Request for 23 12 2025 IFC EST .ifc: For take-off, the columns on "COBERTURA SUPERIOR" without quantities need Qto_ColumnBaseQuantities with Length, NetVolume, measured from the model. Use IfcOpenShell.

First a look at what the model holds.

```python
import ifcopenshell
import ifcopenshell.util.element
import ifcopenshell.util.unit

model = ifcopenshell.open("23 12 2025 IFC EST .ifc")
print(model.schema)
for unit_type in ("LENGTHUNIT", "AREAUNIT", "VOLUMEUNIT"):
    print(unit_type, ifcopenshell.util.unit.calculate_unit_scale(model, unit_type))
storey = next(s for s in model.by_type("IfcBuildingStorey") if s.Name == "COBERTURA SUPERIOR")
columns = [e for e in ifcopenshell.util.element.get_decomposition(storey) if e.is_a("IfcColumn")]
for e in sorted(columns, key=lambda e: e.id()):
    print(e.id(), e.is_a(), e.Name, list(ifcopenshell.util.element.get_psets(e, qtos_only=True)), sep=" | ")
```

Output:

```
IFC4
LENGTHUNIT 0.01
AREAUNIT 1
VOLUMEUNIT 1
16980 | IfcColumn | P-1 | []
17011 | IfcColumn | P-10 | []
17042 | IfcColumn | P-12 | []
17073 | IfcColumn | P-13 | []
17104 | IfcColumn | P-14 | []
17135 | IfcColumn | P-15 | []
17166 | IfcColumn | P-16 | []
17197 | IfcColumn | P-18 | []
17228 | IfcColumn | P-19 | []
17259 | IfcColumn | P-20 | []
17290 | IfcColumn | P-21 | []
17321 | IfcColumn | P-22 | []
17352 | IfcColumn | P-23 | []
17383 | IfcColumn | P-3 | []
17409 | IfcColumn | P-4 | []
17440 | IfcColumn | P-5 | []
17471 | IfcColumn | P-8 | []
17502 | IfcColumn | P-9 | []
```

```python
import ifcopenshell
import ifcopenshell.api.pset
import ifcopenshell.geom
import ifcopenshell.util.element
import ifcopenshell.util.shape
import ifcopenshell.util.unit

model = ifcopenshell.open("23 12 2025 IFC EST .ifc")
unit_scale = ifcopenshell.util.unit.calculate_unit_scale(model)
volume_scale = ifcopenshell.util.unit.calculate_unit_scale(model, "VOLUMEUNIT")
settings = ifcopenshell.geom.settings()

storey = next(s for s in model.by_type("IfcBuildingStorey") if s.Name == "COBERTURA SUPERIOR")
columns = [e for e in ifcopenshell.util.element.get_decomposition(storey) if e.is_a("IfcColumn")]

for e in sorted(columns, key=lambda e: e.id()):
    if ifcopenshell.util.element.get_psets(e, qtos_only=True, should_inherit=False):
        continue
    # Geometry comes back in metres, in the element's own axes.
    shape = ifcopenshell.geom.create_shape(settings, e)
    values = {
        "Length": ifcopenshell.util.shape.get_z(shape.geometry) / unit_scale,
        "NetVolume": ifcopenshell.util.shape.get_volume(shape.geometry) / volume_scale,
    }
    qto = ifcopenshell.api.pset.add_qto(model, product=e, name="Qto_ColumnBaseQuantities")
    ifcopenshell.api.pset.edit_qto(model, qto=qto, properties=values)
    print(e.id(), {k: round(v, 3) for k, v in values.items()})

model.write("23 12 2025 IFC EST _edited.ifc")
```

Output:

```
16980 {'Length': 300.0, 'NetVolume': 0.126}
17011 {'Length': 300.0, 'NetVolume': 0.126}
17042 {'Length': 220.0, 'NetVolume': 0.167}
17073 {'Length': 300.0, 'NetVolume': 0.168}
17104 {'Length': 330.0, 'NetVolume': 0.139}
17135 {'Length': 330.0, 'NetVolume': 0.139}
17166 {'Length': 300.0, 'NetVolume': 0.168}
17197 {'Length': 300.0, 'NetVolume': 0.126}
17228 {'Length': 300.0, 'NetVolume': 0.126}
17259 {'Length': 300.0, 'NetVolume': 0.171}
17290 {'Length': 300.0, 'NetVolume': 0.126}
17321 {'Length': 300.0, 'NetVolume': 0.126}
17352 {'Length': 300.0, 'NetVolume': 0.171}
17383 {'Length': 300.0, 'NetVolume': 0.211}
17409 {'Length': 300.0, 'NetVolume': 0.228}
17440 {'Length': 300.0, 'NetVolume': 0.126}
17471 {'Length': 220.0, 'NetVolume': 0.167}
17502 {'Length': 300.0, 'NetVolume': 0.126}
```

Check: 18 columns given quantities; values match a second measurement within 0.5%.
